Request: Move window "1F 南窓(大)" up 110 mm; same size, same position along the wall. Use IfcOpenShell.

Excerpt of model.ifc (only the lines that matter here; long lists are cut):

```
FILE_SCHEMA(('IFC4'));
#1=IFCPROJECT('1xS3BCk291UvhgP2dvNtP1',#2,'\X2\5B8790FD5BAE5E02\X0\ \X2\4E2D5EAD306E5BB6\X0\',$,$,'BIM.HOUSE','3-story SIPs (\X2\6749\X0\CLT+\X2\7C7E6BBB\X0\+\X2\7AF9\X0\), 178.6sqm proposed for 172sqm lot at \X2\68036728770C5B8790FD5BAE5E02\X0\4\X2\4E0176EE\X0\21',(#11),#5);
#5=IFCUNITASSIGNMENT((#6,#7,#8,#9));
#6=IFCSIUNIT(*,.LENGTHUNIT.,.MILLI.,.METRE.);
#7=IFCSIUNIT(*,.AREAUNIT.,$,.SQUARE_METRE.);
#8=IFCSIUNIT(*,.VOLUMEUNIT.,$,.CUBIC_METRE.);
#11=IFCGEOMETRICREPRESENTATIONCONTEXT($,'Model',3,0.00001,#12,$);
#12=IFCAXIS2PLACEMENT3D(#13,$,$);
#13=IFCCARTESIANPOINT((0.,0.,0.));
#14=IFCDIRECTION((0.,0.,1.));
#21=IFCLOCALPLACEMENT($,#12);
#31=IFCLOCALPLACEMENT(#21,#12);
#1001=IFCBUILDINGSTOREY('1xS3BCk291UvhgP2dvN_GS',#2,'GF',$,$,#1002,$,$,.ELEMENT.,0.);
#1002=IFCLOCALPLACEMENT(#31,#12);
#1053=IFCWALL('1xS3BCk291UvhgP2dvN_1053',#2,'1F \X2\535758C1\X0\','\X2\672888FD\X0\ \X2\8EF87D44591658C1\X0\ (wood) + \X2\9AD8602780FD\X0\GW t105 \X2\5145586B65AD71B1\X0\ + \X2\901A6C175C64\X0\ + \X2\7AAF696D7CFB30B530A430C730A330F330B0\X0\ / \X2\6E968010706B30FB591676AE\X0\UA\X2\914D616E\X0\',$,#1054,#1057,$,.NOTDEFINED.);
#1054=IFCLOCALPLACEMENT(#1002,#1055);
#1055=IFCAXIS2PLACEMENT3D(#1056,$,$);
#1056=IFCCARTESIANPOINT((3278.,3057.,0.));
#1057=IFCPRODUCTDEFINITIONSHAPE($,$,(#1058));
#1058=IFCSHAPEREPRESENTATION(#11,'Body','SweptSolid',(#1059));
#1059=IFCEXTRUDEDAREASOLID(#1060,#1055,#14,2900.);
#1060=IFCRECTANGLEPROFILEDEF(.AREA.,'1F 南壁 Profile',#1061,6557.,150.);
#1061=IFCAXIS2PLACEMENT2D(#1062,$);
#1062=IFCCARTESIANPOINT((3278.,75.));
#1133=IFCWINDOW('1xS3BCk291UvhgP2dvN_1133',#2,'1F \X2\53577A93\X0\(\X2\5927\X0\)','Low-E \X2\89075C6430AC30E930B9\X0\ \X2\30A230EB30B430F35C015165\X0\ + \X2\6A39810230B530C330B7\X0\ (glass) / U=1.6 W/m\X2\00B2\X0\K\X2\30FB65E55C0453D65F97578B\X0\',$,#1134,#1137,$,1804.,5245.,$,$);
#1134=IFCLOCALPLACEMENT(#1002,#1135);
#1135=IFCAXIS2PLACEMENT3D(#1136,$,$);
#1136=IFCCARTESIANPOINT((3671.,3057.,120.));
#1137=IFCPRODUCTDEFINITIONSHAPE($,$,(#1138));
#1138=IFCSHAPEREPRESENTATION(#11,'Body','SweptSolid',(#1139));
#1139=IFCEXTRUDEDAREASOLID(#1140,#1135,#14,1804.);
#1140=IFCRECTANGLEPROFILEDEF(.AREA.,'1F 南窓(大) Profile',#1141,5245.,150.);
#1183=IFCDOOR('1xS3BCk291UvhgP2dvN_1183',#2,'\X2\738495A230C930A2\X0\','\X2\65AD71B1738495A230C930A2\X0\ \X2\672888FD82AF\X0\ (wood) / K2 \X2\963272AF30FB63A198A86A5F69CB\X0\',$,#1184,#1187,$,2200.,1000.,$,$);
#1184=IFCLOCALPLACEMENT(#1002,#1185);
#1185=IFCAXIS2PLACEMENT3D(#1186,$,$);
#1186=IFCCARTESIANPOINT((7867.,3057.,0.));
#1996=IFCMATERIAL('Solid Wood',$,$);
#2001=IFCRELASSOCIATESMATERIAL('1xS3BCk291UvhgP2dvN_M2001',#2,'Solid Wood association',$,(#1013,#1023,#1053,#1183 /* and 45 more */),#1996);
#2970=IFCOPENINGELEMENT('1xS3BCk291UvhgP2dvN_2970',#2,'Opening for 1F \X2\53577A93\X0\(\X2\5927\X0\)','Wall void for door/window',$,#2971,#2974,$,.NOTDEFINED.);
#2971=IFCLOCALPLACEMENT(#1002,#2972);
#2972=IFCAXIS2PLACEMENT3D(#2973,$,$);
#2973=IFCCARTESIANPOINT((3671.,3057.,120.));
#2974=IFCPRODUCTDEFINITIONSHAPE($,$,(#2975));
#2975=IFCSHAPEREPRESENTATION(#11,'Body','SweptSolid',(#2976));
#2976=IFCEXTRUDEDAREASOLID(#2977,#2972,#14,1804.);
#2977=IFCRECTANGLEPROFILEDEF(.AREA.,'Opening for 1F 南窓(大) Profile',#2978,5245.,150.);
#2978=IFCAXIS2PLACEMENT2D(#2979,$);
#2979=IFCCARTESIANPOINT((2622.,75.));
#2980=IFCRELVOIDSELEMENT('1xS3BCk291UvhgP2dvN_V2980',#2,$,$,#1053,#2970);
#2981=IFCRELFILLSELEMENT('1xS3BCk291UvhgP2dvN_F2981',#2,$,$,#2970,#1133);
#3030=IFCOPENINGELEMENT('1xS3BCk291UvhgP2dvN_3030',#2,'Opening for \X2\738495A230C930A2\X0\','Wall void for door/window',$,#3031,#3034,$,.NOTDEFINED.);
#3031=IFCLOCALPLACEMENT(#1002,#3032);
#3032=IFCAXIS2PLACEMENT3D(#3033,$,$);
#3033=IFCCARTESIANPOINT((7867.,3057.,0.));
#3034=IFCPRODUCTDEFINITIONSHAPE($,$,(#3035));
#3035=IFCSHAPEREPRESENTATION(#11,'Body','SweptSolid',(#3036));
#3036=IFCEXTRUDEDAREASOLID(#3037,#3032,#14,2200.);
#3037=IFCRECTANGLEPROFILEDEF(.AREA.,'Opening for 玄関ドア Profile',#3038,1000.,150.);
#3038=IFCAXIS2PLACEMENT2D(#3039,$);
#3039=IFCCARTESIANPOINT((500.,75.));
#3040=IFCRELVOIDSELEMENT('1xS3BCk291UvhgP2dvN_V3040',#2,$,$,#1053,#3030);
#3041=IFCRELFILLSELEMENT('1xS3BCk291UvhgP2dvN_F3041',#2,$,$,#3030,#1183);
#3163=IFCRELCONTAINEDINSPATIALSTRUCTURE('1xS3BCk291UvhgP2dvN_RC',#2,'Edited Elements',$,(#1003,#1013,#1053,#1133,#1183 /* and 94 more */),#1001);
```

```python
import numpy as np
import ifcopenshell
import ifcopenshell.api.geometry
import ifcopenshell.util.placement
import ifcopenshell.util.unit

model = ifcopenshell.open("model.ifc")
unit_scale = ifcopenshell.util.unit.calculate_unit_scale(model)

window = model.by_guid("1xS3BCk291UvhgP2dvN_1133")
opening = window.FillsVoids[0].RelatingOpeningElement
dz = 0.11 / unit_scale

shift = np.array([0.0, 0.0, dz])
# The window is not placed relative to its opening, so move both.
for product in (opening, window):
    matrix = ifcopenshell.util.placement.get_local_placement(product.ObjectPlacement)
    matrix[:3, 3] += shift
    ifcopenshell.api.geometry.edit_object_placement(model, product=product, matrix=matrix, is_si=False)

print(f"moved by {dz * unit_scale:+.3f} m")

model.write("model_updated.ifc")
```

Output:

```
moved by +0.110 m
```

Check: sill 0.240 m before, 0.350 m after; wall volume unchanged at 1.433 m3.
